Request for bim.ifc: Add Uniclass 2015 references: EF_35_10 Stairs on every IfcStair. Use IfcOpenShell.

First a look at what the model holds.

```python
import ifcopenshell

model = ifcopenshell.open("bim.ifc")
print(model.schema)
print("classifications:", [c.Name for c in model.by_type("IfcClassification")])
for ifc_class in ("IfcDoor", "IfcRoof", "IfcStair", "IfcWall", "IfcWindow"):
    print(ifc_class, len(model.by_type(ifc_class)))
```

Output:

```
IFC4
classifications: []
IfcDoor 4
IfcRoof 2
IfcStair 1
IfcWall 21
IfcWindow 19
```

```python
import ifcopenshell
import ifcopenshell.api.classification

model = ifcopenshell.open("bim.ifc")

system = ifcopenshell.api.classification.add_classification(model, classification="Uniclass 2015")

codes = {
    "IfcStair": ("EF_35_10", "Stairs"),
}
for ifc_class, (code, name) in codes.items():
    products = model.by_type(ifc_class)
    ifcopenshell.api.classification.add_reference(
        model, products=products, classification=system, identification=code, name=name
    )
    print(code, len(products))

model.write("bim_updated.ifc")
```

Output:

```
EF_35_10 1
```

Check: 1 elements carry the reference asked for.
